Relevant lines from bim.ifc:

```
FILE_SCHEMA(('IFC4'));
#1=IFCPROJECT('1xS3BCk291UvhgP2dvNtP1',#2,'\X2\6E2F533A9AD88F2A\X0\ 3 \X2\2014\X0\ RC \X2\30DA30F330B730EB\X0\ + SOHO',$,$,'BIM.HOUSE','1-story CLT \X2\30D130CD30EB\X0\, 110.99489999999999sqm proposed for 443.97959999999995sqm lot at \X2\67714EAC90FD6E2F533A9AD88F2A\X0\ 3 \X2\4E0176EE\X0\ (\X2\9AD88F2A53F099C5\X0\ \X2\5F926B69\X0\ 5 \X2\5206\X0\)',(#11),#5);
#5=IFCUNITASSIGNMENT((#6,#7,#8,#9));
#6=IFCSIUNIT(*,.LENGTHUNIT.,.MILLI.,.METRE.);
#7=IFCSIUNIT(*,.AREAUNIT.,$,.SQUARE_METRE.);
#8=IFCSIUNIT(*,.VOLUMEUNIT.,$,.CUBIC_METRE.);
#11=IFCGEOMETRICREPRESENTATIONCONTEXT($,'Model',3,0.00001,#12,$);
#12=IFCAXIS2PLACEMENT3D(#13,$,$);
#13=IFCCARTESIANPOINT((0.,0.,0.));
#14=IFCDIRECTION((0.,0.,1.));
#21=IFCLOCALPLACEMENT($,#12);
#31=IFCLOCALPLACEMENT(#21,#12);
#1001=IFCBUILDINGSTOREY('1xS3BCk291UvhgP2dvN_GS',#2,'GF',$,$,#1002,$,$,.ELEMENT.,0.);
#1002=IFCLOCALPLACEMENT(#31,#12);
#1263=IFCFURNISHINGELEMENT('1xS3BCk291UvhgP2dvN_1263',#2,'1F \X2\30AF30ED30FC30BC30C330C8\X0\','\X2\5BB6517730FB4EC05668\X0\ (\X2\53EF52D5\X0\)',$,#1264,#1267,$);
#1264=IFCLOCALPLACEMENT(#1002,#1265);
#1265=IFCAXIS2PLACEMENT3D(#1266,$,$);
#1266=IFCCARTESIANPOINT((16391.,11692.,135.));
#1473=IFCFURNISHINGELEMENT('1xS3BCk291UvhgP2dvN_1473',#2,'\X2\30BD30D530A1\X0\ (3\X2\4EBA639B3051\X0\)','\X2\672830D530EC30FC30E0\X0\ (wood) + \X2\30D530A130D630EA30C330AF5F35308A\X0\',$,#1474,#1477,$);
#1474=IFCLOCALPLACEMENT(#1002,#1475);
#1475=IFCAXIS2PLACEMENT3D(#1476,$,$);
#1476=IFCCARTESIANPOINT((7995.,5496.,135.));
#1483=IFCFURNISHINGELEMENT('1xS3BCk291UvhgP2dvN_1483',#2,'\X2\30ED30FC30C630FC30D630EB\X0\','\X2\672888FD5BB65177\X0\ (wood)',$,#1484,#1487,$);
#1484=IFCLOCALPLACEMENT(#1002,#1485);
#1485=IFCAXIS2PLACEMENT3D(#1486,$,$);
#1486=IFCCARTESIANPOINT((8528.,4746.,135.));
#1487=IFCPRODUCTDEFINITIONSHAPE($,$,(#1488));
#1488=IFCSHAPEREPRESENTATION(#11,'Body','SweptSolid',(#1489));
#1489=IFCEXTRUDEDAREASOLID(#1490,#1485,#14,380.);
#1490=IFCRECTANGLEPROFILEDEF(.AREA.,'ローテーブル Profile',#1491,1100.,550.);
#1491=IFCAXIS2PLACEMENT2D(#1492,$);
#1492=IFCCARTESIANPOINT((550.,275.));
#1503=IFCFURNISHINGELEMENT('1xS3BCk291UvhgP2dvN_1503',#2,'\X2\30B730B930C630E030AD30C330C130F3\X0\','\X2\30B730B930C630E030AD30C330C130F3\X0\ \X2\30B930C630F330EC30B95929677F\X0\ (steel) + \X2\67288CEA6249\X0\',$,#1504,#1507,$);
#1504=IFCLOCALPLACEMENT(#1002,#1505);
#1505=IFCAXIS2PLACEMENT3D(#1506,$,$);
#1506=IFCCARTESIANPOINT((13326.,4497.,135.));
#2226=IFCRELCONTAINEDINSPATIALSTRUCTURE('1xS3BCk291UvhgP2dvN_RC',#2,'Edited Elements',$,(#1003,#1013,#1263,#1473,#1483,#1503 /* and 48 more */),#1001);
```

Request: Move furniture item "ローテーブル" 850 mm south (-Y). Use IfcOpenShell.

```python
import ifcopenshell
import ifcopenshell.api.geometry
import ifcopenshell.util.placement

model = ifcopenshell.open("bim.ifc")

item = model.by_guid("1xS3BCk291UvhgP2dvN_1483")
matrix = ifcopenshell.util.placement.get_local_placement(item.ObjectPlacement)
matrix[1, 3] -= 850.0
ifcopenshell.api.geometry.edit_object_placement(model, product=item, matrix=matrix, is_si=False)

print(ifcopenshell.util.placement.get_local_placement(item.ObjectPlacement).round(3) + 0.0)

model.write("bim-out.ifc")
```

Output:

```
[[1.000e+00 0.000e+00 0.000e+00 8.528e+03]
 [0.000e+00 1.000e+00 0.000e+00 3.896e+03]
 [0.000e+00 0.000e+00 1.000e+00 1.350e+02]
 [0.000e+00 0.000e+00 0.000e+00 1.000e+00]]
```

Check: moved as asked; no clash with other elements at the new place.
